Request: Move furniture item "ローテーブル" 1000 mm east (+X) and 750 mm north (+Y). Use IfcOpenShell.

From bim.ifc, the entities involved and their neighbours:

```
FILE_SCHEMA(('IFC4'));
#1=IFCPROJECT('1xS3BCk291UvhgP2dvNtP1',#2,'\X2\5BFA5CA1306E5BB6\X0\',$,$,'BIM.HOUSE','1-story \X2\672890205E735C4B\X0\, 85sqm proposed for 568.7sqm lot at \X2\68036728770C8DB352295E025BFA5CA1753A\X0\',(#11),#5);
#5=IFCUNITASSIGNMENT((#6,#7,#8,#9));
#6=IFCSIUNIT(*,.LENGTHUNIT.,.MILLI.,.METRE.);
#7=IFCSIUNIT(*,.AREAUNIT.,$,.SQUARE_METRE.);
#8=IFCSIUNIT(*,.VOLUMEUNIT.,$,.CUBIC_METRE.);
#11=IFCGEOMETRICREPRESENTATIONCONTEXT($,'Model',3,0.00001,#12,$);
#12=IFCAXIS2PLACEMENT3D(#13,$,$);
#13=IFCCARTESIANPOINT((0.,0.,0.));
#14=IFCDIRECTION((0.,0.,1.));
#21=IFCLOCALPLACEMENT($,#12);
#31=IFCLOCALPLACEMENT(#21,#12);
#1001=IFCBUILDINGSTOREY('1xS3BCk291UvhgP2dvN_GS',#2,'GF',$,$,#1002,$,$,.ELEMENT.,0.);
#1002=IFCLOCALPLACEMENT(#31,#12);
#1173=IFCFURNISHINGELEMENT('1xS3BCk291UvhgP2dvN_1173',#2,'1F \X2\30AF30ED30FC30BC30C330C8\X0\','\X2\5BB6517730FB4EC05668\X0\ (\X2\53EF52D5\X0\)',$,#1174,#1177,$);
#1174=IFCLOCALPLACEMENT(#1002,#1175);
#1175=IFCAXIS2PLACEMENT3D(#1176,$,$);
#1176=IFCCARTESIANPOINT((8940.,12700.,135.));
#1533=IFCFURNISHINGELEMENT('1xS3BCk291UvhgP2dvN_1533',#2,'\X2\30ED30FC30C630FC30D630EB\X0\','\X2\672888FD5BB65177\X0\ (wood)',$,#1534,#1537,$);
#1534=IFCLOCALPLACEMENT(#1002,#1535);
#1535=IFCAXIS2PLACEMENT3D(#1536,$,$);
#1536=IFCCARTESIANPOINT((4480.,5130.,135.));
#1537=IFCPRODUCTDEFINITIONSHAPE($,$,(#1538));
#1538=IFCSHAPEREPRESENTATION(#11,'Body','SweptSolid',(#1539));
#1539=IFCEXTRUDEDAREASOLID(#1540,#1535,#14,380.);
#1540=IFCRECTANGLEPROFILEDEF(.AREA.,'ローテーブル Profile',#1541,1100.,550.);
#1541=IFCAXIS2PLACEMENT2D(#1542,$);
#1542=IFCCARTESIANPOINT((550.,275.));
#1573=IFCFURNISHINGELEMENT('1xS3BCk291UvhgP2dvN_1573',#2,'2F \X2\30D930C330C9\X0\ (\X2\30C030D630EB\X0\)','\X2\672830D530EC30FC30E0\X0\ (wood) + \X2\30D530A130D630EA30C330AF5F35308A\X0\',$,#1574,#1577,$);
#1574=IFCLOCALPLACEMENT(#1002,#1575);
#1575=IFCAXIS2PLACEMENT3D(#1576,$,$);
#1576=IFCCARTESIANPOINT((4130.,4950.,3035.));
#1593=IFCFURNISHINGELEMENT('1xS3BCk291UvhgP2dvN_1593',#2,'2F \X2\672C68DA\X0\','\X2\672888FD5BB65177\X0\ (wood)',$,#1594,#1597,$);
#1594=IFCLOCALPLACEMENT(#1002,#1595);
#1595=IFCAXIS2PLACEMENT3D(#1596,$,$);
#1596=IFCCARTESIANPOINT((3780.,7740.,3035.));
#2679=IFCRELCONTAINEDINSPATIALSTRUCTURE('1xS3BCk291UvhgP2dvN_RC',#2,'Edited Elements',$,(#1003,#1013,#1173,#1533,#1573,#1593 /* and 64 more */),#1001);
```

```python
import ifcopenshell
import ifcopenshell.api.geometry
import ifcopenshell.util.placement
import ifcopenshell.util.unit

model = ifcopenshell.open("bim.ifc")
unit_scale = ifcopenshell.util.unit.calculate_unit_scale(model)

item = model.by_id(1533)
matrix = ifcopenshell.util.placement.get_local_placement(item.ObjectPlacement)
matrix[0, 3] += 1 / unit_scale
matrix[1, 3] += 0.75 / unit_scale
ifcopenshell.api.geometry.edit_object_placement(model, product=item, matrix=matrix, is_si=False)

print(ifcopenshell.util.placement.get_local_placement(item.ObjectPlacement).round(3) + 0.0)

model.write("bim_v2.ifc")
```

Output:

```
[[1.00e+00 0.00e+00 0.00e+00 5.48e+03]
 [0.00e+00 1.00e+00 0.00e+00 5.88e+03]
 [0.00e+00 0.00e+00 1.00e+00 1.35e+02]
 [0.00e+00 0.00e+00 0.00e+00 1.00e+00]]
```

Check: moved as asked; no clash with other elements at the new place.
